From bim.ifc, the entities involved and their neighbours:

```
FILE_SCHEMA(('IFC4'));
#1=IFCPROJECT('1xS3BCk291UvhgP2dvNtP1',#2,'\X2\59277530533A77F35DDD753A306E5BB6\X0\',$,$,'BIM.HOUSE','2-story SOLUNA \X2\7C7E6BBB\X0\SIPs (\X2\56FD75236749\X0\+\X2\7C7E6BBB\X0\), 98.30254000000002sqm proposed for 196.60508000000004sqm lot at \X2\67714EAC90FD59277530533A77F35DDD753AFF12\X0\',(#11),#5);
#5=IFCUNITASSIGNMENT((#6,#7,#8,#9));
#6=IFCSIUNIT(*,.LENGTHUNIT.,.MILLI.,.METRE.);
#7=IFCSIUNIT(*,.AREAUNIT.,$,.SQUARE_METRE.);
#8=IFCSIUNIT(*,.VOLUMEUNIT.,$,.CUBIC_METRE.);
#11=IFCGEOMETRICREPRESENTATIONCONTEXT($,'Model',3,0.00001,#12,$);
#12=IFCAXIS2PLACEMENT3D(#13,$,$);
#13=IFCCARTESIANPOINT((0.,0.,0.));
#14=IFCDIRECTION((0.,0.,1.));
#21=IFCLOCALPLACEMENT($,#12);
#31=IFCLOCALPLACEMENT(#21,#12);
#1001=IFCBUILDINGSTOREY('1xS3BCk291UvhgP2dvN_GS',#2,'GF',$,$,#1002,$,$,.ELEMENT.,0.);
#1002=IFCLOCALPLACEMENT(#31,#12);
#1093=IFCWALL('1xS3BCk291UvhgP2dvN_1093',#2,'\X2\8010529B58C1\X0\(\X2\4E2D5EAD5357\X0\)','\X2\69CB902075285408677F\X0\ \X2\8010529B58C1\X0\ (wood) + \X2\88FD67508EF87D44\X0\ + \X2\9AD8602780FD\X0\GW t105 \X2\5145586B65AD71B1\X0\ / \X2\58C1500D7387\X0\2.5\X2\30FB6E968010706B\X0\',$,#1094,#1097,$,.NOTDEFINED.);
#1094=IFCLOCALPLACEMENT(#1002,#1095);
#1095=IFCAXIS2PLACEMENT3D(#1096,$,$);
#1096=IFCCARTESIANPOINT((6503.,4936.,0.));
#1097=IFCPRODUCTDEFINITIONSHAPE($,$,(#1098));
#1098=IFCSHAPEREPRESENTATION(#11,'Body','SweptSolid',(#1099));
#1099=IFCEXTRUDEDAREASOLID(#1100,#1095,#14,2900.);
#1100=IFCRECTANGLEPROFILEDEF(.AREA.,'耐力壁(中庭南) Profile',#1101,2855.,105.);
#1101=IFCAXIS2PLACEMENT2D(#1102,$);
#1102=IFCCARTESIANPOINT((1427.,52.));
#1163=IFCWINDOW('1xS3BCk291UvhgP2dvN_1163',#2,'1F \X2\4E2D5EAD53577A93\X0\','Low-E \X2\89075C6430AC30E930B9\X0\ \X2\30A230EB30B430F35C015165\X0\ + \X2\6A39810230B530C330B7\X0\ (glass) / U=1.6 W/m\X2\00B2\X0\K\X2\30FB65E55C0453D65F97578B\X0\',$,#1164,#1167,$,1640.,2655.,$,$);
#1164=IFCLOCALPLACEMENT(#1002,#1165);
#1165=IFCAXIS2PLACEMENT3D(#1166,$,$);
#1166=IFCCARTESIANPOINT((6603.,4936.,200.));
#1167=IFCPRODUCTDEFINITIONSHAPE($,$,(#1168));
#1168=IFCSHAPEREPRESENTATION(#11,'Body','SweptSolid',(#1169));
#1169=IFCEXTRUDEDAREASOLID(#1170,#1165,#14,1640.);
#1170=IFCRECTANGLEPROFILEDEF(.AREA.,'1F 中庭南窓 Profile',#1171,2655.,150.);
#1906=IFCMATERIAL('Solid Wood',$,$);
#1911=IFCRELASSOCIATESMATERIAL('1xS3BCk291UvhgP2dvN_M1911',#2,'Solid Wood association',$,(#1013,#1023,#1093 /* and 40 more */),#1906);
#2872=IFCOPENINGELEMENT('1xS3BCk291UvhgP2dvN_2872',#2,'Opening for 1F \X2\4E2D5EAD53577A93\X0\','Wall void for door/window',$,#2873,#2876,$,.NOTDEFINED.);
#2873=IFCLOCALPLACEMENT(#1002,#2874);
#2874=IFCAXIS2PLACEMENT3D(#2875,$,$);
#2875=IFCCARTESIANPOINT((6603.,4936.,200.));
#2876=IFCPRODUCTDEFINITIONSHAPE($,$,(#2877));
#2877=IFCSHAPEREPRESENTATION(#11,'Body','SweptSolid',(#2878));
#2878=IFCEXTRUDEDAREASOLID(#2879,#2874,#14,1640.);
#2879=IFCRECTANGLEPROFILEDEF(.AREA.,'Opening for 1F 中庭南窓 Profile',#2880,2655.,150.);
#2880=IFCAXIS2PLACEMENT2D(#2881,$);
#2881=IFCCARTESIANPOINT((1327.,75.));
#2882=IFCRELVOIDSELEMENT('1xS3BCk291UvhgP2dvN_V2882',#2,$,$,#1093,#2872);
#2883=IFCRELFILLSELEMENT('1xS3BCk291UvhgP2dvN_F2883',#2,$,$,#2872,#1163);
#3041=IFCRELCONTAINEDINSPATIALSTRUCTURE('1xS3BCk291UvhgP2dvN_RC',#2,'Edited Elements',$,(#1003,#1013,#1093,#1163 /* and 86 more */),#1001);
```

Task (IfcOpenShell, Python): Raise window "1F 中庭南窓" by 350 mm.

```python
import numpy as np
import ifcopenshell
import ifcopenshell.api.geometry
import ifcopenshell.util.placement
import ifcopenshell.util.unit

model = ifcopenshell.open("bim.ifc")
unit_scale = ifcopenshell.util.unit.calculate_unit_scale(model)

window = model.by_guid("1xS3BCk291UvhgP2dvN_1163")
opening = window.FillsVoids[0].RelatingOpeningElement
dz = 350.0

shift = np.array([0.0, 0.0, dz])
# The window is not placed relative to its opening, so move both.
for product in (opening, window):
    matrix = ifcopenshell.util.placement.get_local_placement(product.ObjectPlacement)
    matrix[:3, 3] += shift
    ifcopenshell.api.geometry.edit_object_placement(model, product=product, matrix=matrix, is_si=False)

print(f"moved by {dz * unit_scale:+.3f} m")

model.write("bim_rev.ifc")
```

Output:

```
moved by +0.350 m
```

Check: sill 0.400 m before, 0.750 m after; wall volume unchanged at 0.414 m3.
